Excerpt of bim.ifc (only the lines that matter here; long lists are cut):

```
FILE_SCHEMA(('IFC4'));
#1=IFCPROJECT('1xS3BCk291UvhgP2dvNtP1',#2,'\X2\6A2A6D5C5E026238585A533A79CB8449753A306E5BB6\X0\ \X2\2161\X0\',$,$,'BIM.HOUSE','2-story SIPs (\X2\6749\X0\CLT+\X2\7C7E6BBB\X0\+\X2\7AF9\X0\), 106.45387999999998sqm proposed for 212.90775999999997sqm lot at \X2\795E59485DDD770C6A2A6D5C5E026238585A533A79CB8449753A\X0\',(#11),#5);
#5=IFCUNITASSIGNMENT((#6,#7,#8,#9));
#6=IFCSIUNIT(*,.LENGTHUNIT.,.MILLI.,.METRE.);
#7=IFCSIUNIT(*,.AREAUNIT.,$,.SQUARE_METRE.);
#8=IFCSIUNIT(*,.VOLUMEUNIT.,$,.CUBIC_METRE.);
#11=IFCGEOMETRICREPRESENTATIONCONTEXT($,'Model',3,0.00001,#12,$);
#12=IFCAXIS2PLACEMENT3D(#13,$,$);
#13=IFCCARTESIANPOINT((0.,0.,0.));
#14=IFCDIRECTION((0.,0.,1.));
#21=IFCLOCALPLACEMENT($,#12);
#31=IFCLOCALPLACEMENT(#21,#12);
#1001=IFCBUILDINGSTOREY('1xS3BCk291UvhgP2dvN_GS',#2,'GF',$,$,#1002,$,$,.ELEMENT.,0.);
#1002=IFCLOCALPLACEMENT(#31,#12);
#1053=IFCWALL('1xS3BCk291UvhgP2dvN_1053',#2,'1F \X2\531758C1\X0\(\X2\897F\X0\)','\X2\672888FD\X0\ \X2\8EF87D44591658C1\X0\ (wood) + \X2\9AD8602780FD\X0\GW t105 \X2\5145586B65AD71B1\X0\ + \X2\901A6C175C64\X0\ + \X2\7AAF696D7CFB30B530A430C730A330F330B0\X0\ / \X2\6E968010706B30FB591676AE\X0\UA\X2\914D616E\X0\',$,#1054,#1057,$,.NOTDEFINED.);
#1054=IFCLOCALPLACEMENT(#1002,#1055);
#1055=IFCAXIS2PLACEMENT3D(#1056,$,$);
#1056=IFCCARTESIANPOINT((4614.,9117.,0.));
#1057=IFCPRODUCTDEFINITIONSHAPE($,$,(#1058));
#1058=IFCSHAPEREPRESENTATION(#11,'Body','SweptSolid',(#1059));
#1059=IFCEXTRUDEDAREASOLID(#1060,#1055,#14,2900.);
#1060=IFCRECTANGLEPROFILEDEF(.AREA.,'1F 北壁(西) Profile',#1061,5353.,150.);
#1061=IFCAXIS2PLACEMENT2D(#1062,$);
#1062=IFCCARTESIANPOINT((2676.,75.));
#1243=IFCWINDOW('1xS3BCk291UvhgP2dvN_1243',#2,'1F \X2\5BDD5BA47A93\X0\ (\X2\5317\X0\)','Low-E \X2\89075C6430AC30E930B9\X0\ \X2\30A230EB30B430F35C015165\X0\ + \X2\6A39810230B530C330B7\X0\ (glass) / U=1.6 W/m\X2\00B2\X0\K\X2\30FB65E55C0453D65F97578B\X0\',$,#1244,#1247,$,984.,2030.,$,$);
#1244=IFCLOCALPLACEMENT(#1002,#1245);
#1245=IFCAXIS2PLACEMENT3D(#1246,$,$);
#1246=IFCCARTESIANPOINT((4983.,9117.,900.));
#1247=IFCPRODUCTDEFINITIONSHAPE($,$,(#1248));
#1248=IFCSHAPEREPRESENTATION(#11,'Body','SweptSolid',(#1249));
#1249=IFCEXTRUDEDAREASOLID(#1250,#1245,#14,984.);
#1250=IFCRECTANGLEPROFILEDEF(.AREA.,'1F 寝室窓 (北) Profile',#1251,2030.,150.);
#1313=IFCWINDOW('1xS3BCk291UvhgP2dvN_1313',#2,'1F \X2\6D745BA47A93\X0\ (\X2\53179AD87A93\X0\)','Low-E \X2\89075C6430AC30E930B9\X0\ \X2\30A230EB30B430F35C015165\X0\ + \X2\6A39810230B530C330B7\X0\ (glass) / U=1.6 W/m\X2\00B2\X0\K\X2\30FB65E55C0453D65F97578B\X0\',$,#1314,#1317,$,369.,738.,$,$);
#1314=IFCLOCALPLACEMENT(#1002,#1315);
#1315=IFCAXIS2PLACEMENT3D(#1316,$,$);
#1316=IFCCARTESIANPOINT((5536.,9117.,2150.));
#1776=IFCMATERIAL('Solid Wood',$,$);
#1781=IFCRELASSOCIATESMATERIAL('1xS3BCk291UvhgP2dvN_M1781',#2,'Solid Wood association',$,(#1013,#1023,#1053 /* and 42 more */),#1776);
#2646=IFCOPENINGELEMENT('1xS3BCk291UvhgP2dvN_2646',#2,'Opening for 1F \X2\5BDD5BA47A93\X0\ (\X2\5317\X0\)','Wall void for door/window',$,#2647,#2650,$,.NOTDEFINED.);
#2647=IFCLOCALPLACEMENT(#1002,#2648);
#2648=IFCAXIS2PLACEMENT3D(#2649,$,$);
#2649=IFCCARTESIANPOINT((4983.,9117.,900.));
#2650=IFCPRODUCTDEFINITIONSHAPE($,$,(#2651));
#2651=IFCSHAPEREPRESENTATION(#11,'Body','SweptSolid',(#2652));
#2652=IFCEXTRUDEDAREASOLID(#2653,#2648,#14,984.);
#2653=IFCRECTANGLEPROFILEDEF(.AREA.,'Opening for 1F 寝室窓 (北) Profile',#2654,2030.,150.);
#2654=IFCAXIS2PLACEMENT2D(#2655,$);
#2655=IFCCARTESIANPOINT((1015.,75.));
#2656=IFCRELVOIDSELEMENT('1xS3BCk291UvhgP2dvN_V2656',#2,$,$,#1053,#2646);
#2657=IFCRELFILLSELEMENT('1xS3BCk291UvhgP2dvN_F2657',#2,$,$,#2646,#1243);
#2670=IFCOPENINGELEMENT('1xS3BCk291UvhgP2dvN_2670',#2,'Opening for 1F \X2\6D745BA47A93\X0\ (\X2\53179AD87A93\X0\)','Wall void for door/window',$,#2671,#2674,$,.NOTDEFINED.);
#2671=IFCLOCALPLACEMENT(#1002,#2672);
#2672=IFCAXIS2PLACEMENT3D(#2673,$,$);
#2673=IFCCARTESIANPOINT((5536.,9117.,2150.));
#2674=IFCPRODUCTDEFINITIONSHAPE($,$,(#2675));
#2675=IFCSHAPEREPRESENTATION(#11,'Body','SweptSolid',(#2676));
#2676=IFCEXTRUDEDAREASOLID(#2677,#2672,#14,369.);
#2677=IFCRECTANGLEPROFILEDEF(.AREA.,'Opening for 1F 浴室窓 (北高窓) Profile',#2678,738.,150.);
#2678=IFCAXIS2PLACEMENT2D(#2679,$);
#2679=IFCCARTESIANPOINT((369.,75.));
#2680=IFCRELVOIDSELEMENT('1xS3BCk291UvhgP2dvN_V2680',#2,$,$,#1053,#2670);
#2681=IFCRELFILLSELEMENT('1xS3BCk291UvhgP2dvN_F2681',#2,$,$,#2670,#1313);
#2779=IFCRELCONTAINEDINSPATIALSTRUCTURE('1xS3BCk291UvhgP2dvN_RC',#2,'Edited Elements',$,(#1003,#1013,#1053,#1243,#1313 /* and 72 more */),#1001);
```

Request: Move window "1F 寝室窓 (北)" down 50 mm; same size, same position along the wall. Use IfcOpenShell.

```python
import numpy as np
import ifcopenshell
import ifcopenshell.api.geometry
import ifcopenshell.util.placement
import ifcopenshell.util.unit

model = ifcopenshell.open("bim.ifc")
unit_scale = ifcopenshell.util.unit.calculate_unit_scale(model)

window = model.by_guid("1xS3BCk291UvhgP2dvN_1243")
opening = window.FillsVoids[0].RelatingOpeningElement
dz = -0.05 / unit_scale

shift = np.array([0.0, 0.0, dz])
# The window is not placed relative to its opening, so move both.
for product in (opening, window):
    matrix = ifcopenshell.util.placement.get_local_placement(product.ObjectPlacement)
    matrix[:3, 3] += shift
    ifcopenshell.api.geometry.edit_object_placement(model, product=product, matrix=matrix, is_si=False)

print(f"moved by {dz * unit_scale:+.3f} m")

model.write("bim_edited.ifc")
```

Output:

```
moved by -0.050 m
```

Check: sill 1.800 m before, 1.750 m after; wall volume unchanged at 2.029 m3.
